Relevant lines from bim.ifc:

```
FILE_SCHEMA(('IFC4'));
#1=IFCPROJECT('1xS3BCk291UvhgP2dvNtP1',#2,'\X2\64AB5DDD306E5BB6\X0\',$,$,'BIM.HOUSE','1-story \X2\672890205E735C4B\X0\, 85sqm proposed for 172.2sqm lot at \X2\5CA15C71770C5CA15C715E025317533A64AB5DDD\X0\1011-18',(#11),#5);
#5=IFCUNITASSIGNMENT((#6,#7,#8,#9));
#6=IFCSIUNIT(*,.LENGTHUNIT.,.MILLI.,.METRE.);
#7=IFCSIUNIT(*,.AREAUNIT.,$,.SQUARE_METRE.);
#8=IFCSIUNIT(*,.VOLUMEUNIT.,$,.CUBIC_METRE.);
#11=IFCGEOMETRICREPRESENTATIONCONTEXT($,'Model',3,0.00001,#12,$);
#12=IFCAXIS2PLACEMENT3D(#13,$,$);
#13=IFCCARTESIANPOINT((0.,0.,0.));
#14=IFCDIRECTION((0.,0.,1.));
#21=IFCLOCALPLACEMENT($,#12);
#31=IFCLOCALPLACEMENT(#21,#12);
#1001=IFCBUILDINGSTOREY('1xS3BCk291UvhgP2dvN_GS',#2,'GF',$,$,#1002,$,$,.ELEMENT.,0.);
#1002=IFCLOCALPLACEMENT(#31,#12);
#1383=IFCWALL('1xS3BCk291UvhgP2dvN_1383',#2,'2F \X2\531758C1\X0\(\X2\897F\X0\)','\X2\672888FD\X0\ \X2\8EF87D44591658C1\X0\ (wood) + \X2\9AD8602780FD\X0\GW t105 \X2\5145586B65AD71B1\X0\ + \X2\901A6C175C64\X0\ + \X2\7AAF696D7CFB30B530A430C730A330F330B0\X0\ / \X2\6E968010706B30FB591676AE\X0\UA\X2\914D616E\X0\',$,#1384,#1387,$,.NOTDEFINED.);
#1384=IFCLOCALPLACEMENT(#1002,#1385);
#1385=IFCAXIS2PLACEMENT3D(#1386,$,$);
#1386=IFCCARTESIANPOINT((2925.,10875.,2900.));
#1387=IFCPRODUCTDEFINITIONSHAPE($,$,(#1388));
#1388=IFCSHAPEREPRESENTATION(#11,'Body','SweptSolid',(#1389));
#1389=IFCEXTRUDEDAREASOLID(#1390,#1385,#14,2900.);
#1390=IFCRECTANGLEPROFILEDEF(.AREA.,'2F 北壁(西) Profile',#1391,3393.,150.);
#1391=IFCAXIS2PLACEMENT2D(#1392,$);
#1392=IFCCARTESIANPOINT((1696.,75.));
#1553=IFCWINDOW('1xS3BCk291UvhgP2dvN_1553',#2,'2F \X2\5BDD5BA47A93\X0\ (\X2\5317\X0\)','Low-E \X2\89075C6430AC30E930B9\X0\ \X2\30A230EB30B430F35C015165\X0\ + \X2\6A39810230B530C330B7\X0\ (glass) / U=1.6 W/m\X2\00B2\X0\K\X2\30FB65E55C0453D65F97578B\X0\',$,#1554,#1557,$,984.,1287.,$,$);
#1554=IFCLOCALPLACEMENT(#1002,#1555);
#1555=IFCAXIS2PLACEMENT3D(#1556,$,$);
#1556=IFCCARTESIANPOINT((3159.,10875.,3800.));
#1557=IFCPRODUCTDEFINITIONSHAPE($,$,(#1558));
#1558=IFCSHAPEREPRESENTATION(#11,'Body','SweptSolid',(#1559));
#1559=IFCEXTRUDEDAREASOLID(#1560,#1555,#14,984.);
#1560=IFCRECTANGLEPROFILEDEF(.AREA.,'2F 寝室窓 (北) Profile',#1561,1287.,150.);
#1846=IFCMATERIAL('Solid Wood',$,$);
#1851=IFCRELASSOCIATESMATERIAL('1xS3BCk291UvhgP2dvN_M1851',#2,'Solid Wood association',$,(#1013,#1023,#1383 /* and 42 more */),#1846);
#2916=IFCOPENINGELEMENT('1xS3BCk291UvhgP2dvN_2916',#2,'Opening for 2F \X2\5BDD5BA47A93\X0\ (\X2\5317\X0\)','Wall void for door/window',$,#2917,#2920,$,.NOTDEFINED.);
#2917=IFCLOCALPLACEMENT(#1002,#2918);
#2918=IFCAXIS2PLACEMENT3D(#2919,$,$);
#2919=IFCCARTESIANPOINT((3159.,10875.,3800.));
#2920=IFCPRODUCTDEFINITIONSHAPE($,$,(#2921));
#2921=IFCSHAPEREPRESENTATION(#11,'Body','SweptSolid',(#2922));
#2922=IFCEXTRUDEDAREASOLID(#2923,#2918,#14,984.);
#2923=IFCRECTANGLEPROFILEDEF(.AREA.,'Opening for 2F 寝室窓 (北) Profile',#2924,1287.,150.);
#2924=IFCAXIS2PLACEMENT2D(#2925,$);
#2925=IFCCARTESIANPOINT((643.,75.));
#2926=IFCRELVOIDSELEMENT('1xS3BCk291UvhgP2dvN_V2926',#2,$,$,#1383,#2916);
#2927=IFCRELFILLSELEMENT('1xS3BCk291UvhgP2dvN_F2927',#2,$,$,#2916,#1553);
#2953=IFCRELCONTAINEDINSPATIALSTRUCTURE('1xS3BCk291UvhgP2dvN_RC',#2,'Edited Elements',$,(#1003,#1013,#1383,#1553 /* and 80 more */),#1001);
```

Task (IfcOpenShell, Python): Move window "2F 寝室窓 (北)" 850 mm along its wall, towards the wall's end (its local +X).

```python
import ifcopenshell
import ifcopenshell.api.geometry
import ifcopenshell.util.placement

model = ifcopenshell.open("bim.ifc")

window = model.by_guid("1xS3BCk291UvhgP2dvN_1553")
opening = window.FillsVoids[0].RelatingOpeningElement
wall = opening.VoidsElements[0].RelatingBuildingElement

wall_matrix = ifcopenshell.util.placement.get_local_placement(wall.ObjectPlacement)
shift = wall_matrix[:3, 0] * 850.0
before = ifcopenshell.util.placement.get_local_placement(window.ObjectPlacement)[:3, 3].copy()

# The window is not placed relative to its opening, so move both.
for product in (opening, window):
    matrix = ifcopenshell.util.placement.get_local_placement(product.ObjectPlacement)
    matrix[:3, 3] += shift
    ifcopenshell.api.geometry.edit_object_placement(model, product=product, matrix=matrix, is_si=False)

after = ifcopenshell.util.placement.get_local_placement(window.ObjectPlacement)[:3, 3]
print("window moved by", (after - before).round(3) + 0.0)

model.write("bim_v2.ifc")
```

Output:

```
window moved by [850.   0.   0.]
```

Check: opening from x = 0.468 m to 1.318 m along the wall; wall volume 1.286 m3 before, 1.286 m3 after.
